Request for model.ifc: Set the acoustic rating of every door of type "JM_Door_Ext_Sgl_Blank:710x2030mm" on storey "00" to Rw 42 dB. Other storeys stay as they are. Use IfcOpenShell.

First a look at what the model holds.

```python
import ifcopenshell
import ifcopenshell.util.element

model = ifcopenshell.open("model.ifc")
print(model.schema)
storey = next(s for s in model.by_type("IfcBuildingStorey") if s.Name == "00")
doors = [e for e in ifcopenshell.util.element.get_decomposition(storey) if e.is_a("IfcDoor")]
seen = {}
for e in doors:
    element_type = ifcopenshell.util.element.get_type(e)
    key = (element_type.Name if element_type != e and element_type else None, ifcopenshell.util.element.get_pset(e, "Pset_DoorCommon", "AcousticRating"))
    seen[key] = seen.get(key, 0) + 1
for (name, value), count in sorted(seen.items(), key=str):
    print(count, "x", name, "|", value)
```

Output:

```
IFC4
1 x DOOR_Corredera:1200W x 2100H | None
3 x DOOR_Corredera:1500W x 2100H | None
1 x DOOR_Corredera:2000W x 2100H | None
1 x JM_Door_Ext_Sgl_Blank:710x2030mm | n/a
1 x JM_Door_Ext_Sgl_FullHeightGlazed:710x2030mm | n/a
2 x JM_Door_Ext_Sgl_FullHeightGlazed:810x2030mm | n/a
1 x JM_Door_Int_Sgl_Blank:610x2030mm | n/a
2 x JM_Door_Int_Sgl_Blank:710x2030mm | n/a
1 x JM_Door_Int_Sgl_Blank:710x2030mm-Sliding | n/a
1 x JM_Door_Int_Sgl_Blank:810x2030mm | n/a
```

```python
import ifcopenshell
import ifcopenshell.api.pset
import ifcopenshell.util.element

model = ifcopenshell.open("model.ifc")

storey = next(s for s in model.by_type("IfcBuildingStorey") if s.Name == "00")
doors = [e for e in ifcopenshell.util.element.get_decomposition(storey) if e.is_a("IfcDoor")]

count = 0
for e in doors:
    element_type = ifcopenshell.util.element.get_type(e)
    if element_type in (None, e) or element_type.Name != "JM_Door_Ext_Sgl_Blank:710x2030mm":
        continue
    # add_pset returns the element's existing set when there is one.
    pset = ifcopenshell.api.pset.add_pset(model, product=e, name="Pset_DoorCommon")
    ifcopenshell.api.pset.edit_pset(model, pset=pset, properties={"AcousticRating": "Rw 42 dB"})
    count += 1

print(count, "doors updated")

model.write("model_v2.ifc")
```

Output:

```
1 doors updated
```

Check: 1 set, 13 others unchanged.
